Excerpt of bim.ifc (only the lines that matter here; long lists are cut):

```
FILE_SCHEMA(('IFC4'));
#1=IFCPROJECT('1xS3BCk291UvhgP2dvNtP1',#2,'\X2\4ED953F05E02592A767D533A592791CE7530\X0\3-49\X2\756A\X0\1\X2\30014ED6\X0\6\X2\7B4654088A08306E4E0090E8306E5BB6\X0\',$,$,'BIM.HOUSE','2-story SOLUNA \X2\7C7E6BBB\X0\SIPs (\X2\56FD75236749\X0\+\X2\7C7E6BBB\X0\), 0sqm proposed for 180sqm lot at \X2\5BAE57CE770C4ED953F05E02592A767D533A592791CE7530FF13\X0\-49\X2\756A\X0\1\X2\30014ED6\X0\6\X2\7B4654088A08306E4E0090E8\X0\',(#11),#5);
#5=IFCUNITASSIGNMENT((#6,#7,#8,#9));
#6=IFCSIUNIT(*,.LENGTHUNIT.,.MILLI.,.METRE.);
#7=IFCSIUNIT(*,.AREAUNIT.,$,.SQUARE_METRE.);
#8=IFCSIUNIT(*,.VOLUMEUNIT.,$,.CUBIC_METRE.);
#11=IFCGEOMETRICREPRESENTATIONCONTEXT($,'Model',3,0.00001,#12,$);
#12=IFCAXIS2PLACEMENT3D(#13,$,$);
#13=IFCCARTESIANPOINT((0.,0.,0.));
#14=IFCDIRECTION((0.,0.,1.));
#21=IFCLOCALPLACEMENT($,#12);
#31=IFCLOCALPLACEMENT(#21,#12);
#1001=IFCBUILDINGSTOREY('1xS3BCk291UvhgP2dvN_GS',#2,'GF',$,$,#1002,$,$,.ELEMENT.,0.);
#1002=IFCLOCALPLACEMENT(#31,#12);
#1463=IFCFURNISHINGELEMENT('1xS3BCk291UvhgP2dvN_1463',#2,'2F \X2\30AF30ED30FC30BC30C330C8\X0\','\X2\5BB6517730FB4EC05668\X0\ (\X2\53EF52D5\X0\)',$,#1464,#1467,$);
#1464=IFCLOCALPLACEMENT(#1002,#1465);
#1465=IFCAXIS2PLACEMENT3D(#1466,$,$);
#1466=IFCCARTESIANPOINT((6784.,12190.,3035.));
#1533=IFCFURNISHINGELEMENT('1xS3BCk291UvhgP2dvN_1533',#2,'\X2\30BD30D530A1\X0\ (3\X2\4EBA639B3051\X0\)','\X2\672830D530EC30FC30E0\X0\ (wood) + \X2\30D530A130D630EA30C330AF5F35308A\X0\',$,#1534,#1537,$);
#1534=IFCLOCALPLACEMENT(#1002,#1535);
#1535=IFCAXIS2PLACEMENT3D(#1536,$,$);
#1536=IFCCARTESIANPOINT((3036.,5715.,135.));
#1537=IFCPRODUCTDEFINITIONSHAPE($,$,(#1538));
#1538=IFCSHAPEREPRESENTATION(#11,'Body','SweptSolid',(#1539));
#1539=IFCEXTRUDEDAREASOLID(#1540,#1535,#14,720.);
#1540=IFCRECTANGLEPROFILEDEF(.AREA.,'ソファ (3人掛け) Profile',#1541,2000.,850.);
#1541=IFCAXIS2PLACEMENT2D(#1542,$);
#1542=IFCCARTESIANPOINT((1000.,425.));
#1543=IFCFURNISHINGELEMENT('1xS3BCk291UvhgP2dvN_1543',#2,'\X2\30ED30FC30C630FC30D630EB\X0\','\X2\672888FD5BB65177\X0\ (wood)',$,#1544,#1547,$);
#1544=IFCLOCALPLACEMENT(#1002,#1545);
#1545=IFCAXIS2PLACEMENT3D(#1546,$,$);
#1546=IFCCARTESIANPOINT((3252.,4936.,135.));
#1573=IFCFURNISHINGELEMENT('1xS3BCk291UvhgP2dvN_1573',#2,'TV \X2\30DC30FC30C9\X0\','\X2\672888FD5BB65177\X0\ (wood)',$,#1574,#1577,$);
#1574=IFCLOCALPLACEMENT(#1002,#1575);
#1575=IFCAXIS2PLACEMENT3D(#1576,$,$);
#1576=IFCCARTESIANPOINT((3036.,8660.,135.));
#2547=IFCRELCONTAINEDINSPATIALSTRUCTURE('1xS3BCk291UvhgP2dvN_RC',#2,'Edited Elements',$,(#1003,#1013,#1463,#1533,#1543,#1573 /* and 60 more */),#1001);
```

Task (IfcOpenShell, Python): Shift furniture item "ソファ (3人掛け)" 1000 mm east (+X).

```python
import ifcopenshell
import ifcopenshell.api.geometry
import ifcopenshell.util.placement
import ifcopenshell.util.unit

model = ifcopenshell.open("bim.ifc")
unit_scale = ifcopenshell.util.unit.calculate_unit_scale(model)

item = model.by_id(1533)
matrix = ifcopenshell.util.placement.get_local_placement(item.ObjectPlacement)
matrix[0, 3] += 1 / unit_scale
ifcopenshell.api.geometry.edit_object_placement(model, product=item, matrix=matrix, is_si=False)

print(ifcopenshell.util.placement.get_local_placement(item.ObjectPlacement).round(3) + 0.0)

model.write("bim_edited.ifc")
```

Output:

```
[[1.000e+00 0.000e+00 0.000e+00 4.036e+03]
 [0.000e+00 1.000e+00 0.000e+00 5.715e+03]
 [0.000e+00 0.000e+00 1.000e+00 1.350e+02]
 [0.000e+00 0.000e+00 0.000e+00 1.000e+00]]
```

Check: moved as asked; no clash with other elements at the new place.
